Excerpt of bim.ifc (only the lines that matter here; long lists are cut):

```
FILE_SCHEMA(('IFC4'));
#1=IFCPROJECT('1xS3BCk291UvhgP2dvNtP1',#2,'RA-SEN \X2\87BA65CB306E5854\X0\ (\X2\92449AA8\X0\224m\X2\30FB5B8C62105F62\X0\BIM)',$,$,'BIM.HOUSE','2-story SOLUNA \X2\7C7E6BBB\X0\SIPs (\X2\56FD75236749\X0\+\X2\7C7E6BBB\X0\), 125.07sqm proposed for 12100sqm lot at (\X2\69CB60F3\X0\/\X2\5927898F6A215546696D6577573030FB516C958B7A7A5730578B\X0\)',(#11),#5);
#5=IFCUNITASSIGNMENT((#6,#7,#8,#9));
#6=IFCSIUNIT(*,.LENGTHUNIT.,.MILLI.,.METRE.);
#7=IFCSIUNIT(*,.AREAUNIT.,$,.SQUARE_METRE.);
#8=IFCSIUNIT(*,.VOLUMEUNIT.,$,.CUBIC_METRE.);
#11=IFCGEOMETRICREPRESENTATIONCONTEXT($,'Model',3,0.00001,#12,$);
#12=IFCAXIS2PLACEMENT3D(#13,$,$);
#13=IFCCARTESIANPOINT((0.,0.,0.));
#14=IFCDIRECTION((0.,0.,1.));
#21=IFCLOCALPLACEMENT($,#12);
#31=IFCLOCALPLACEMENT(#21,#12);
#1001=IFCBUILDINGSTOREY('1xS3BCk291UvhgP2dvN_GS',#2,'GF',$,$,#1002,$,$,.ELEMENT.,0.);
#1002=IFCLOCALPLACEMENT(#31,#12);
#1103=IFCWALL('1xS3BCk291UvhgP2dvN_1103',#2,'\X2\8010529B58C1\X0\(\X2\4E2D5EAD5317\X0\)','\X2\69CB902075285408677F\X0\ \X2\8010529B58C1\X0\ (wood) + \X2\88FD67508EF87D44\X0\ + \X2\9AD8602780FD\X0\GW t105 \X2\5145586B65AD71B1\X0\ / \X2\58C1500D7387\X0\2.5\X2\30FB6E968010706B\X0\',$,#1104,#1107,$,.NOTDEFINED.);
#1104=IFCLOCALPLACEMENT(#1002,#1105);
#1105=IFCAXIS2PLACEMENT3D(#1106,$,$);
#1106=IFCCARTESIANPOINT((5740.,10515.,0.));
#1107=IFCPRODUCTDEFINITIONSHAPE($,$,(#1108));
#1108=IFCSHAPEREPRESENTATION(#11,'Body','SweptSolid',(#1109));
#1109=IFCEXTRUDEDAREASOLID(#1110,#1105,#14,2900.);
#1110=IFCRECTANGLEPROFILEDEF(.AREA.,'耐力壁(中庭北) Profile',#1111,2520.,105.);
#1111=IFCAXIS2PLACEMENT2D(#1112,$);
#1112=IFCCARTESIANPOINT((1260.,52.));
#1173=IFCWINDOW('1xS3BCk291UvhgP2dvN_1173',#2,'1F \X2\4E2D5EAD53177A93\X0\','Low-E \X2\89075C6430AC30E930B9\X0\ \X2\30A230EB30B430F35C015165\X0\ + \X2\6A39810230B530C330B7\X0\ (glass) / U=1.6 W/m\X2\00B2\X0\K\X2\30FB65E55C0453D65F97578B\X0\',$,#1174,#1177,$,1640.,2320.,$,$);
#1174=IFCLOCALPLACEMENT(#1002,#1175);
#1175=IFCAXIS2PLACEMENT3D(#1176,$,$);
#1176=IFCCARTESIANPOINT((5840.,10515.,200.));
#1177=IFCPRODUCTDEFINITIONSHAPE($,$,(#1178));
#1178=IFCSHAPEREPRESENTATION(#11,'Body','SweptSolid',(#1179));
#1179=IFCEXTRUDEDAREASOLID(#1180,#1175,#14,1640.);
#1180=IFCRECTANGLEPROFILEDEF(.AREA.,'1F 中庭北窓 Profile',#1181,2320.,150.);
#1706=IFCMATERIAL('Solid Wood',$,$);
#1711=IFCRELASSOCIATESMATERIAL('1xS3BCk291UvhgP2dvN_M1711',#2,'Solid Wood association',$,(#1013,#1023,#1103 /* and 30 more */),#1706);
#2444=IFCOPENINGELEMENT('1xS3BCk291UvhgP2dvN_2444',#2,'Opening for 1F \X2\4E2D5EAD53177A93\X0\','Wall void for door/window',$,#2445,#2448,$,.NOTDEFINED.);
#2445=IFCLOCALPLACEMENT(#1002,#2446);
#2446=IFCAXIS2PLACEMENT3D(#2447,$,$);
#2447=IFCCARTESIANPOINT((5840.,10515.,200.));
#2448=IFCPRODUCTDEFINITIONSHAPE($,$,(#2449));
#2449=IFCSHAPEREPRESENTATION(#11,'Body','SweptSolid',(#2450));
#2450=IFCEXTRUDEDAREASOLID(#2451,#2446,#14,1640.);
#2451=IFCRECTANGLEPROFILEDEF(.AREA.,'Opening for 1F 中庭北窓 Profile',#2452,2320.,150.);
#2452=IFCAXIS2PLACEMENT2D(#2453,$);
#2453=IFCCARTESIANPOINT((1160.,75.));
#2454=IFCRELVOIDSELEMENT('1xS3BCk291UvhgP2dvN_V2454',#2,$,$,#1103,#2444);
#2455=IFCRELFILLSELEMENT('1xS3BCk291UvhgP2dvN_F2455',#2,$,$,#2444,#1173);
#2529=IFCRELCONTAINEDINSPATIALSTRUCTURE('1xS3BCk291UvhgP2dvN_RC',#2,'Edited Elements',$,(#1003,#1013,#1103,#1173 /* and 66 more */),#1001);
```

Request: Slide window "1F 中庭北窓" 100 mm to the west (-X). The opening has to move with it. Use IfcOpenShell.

```python
import ifcopenshell
import ifcopenshell.api.geometry
import ifcopenshell.util.placement

model = ifcopenshell.open("bim.ifc")

window = model.by_id(1173)
opening = window.FillsVoids[0].RelatingOpeningElement
wall = opening.VoidsElements[0].RelatingBuildingElement

wall_matrix = ifcopenshell.util.placement.get_local_placement(wall.ObjectPlacement)
shift = wall_matrix[:3, 0] * -100.0
before = ifcopenshell.util.placement.get_local_placement(window.ObjectPlacement)[:3, 3].copy()

# The window is not placed relative to its opening, so move both.
for product in (opening, window):
    matrix = ifcopenshell.util.placement.get_local_placement(product.ObjectPlacement)
    matrix[:3, 3] += shift
    ifcopenshell.api.geometry.edit_object_placement(model, product=product, matrix=matrix, is_si=False)

after = ifcopenshell.util.placement.get_local_placement(window.ObjectPlacement)[:3, 3]
print("window moved by", (after - before).round(3) + 0.0)

model.write("bim_v2.ifc")
```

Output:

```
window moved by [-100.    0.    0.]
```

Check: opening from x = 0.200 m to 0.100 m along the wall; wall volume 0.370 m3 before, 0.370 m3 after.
